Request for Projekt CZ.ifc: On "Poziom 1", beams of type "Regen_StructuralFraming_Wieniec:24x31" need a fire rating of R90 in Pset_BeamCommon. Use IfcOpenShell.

First a look at what the model holds.

```python
import ifcopenshell
import ifcopenshell.util.element

model = ifcopenshell.open("Projekt CZ.ifc")
print(model.schema)
storey = next(s for s in model.by_type("IfcBuildingStorey") if s.Name == "Poziom 1")
beams = [e for e in ifcopenshell.util.element.get_decomposition(storey) if e.is_a("IfcBeam")]
seen = {}
for e in beams:
    element_type = ifcopenshell.util.element.get_type(e)
    key = (element_type.Name if element_type != e and element_type else None, ifcopenshell.util.element.get_pset(e, "Pset_BeamCommon", "FireRating"))
    seen[key] = seen.get(key, 0) + 1
for (name, value), count in sorted(seen.items(), key=str):
    print(count, "x", name, "|", value)
```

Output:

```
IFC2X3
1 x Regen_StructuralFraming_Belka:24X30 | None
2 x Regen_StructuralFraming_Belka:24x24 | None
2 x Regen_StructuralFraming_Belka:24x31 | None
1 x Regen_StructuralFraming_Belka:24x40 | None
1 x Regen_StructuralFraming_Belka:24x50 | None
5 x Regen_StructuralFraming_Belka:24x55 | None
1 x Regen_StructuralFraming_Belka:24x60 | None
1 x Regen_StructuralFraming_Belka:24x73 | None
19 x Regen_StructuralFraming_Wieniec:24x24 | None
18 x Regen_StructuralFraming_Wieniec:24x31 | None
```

```python
import ifcopenshell
import ifcopenshell.api.pset
import ifcopenshell.util.element

model = ifcopenshell.open("Projekt CZ.ifc")

storey = next(s for s in model.by_type("IfcBuildingStorey") if s.Name == "Poziom 1")
beams = [e for e in ifcopenshell.util.element.get_decomposition(storey) if e.is_a("IfcBeam")]

count = 0
for e in beams:
    element_type = ifcopenshell.util.element.get_type(e)
    if element_type in (None, e) or element_type.Name != "Regen_StructuralFraming_Wieniec:24x31":
        continue
    # add_pset returns the element's existing set when there is one.
    pset = ifcopenshell.api.pset.add_pset(model, product=e, name="Pset_BeamCommon")
    ifcopenshell.api.pset.edit_pset(model, pset=pset, properties={"FireRating": "R90"})
    count += 1

print(count, "beams updated")

model.write("Projekt CZ_edited.ifc")
```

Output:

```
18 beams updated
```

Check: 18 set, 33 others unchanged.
